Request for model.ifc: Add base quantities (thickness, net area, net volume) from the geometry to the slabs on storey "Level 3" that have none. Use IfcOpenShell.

First a look at what the model holds.

```python
import ifcopenshell
import ifcopenshell.util.element
import ifcopenshell.util.unit

model = ifcopenshell.open("model.ifc")
print(model.schema)
for unit_type in ("LENGTHUNIT", "AREAUNIT", "VOLUMEUNIT"):
    print(unit_type, ifcopenshell.util.unit.calculate_unit_scale(model, unit_type))
storey = next(s for s in model.by_type("IfcBuildingStorey") if s.Name == "Level 3")
slabs = [e for e in ifcopenshell.util.element.get_decomposition(storey) if e.is_a("IfcSlab")]
for e in sorted(slabs, key=lambda e: e.id()):
    print(e.id(), e.is_a(), e.Name, list(ifcopenshell.util.element.get_psets(e, qtos_only=True)), sep=" | ")
```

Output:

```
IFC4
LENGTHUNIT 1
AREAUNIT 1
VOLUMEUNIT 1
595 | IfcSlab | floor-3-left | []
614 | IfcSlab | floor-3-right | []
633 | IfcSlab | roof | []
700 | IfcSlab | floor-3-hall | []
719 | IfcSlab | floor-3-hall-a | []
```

```python
import ifcopenshell
import ifcopenshell.api.pset
import ifcopenshell.geom
import ifcopenshell.util.element
import ifcopenshell.util.shape
import ifcopenshell.util.unit

model = ifcopenshell.open("model.ifc")
unit_scale = ifcopenshell.util.unit.calculate_unit_scale(model)
area_scale = ifcopenshell.util.unit.calculate_unit_scale(model, "AREAUNIT")
volume_scale = ifcopenshell.util.unit.calculate_unit_scale(model, "VOLUMEUNIT")
settings = ifcopenshell.geom.settings()

storey = next(s for s in model.by_type("IfcBuildingStorey") if s.Name == "Level 3")
slabs = [e for e in ifcopenshell.util.element.get_decomposition(storey) if e.is_a("IfcSlab")]

for e in sorted(slabs, key=lambda e: e.id()):
    if ifcopenshell.util.element.get_psets(e, qtos_only=True, should_inherit=False):
        continue
    # Geometry comes back in metres, in the element's own axes.
    shape = ifcopenshell.geom.create_shape(settings, e)
    values = {
        "Width": ifcopenshell.util.shape.get_z(shape.geometry) / unit_scale,
        "NetArea": ifcopenshell.util.shape.get_footprint_area(shape.geometry) / area_scale,
        "NetVolume": ifcopenshell.util.shape.get_volume(shape.geometry) / volume_scale,
    }
    qto = ifcopenshell.api.pset.add_qto(model, product=e, name="Qto_SlabBaseQuantities")
    ifcopenshell.api.pset.edit_qto(model, qto=qto, properties=values)
    print(e.id(), {k: round(v, 3) for k, v in values.items()})

model.write("model_edited.ifc")
```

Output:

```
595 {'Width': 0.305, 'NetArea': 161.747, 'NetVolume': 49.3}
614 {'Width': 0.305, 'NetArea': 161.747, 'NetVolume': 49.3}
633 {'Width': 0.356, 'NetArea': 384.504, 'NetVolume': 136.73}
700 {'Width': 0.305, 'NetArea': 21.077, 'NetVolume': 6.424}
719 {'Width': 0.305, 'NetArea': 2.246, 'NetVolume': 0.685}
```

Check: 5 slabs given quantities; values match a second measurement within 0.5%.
